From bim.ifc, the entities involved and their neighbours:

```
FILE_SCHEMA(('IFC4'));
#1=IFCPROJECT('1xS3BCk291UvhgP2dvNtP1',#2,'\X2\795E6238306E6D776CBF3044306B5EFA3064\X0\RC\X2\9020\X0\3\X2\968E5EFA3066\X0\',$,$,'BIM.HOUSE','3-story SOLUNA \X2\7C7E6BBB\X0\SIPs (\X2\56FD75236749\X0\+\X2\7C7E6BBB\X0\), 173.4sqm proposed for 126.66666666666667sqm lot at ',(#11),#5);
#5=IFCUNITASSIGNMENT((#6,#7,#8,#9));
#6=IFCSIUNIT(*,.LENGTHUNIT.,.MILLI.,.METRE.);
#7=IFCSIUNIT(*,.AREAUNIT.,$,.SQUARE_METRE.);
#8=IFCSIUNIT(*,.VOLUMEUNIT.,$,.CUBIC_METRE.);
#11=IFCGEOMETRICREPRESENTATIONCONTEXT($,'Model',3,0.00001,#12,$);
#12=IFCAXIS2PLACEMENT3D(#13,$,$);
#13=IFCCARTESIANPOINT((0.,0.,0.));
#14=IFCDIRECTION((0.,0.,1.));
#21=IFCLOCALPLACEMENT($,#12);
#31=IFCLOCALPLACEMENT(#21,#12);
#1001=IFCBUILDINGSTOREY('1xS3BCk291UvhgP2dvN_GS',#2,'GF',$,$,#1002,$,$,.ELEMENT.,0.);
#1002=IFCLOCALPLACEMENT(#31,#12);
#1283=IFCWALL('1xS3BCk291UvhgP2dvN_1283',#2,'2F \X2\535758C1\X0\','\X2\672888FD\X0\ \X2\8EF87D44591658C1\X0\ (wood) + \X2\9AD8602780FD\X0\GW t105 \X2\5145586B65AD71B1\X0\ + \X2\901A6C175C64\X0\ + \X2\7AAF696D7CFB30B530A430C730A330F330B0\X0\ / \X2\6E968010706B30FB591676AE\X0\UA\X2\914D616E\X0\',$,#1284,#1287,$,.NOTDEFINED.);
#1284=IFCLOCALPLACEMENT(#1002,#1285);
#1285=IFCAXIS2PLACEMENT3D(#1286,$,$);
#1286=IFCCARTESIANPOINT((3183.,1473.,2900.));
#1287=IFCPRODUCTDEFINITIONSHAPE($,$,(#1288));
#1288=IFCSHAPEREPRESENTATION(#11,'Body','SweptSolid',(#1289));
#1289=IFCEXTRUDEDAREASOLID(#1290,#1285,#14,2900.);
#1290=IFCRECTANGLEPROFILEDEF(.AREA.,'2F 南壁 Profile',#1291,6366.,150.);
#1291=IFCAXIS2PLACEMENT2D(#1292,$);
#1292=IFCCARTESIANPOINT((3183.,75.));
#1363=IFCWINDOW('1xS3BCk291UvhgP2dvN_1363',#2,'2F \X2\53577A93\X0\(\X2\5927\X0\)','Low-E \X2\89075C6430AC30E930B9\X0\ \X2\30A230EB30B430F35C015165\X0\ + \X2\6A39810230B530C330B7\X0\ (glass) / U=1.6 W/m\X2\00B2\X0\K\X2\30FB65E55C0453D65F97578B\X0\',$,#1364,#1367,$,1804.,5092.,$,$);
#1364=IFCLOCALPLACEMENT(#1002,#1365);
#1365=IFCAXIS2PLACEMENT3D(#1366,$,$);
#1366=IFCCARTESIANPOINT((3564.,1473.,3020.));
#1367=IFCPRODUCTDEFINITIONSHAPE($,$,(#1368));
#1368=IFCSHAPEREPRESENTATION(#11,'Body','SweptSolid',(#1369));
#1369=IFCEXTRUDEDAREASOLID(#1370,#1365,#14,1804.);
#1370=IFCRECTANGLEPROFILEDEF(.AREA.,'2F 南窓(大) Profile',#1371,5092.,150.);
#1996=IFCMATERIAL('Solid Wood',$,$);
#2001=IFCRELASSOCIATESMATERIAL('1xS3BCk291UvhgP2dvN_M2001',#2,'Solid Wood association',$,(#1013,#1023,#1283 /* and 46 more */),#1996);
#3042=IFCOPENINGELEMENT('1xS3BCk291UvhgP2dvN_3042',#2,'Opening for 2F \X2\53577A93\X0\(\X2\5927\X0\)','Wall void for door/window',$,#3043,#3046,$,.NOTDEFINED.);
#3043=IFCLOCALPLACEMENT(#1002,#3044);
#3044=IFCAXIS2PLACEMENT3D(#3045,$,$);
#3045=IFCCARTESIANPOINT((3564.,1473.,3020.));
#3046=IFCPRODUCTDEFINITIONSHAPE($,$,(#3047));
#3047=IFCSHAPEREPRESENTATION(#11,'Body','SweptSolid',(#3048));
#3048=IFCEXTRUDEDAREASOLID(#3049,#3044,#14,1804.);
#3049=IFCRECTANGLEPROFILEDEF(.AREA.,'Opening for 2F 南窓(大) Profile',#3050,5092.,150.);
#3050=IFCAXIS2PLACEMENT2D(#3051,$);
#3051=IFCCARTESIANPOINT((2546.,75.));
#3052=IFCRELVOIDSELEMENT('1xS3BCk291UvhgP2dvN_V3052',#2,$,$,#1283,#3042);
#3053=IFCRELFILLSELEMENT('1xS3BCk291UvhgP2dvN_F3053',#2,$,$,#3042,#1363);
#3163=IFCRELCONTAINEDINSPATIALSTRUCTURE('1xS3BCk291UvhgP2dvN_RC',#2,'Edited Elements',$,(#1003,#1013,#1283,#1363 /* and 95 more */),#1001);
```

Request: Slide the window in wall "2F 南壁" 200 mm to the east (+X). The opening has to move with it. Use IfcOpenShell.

```python
import ifcopenshell
import ifcopenshell.api.geometry
import ifcopenshell.util.placement
import ifcopenshell.util.unit

model = ifcopenshell.open("bim.ifc")
unit_scale = ifcopenshell.util.unit.calculate_unit_scale(model)

window = model.by_guid("1xS3BCk291UvhgP2dvN_1363")
opening = window.FillsVoids[0].RelatingOpeningElement
wall = opening.VoidsElements[0].RelatingBuildingElement

wall_matrix = ifcopenshell.util.placement.get_local_placement(wall.ObjectPlacement)
shift = wall_matrix[:3, 0] * 0.2 / unit_scale
before = ifcopenshell.util.placement.get_local_placement(window.ObjectPlacement)[:3, 3].copy()

# The window is not placed relative to its opening, so move both.
for product in (opening, window):
    matrix = ifcopenshell.util.placement.get_local_placement(product.ObjectPlacement)
    matrix[:3, 3] += shift
    ifcopenshell.api.geometry.edit_object_placement(model, product=product, matrix=matrix, is_si=False)

after = ifcopenshell.util.placement.get_local_placement(window.ObjectPlacement)[:3, 3]
print("window moved by", (after - before).round(3) + 0.0)

model.write("bim_updated.ifc")
```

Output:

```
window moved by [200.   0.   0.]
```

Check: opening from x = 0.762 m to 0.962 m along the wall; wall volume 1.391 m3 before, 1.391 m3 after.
